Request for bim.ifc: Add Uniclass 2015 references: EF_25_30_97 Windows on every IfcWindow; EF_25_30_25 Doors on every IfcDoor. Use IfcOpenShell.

First a look at what the model holds.

```python
import ifcopenshell

model = ifcopenshell.open("bim.ifc")
print(model.schema)
print("classifications:", [c.Name for c in model.by_type("IfcClassification")])
for ifc_class in ("IfcDoor", "IfcRoof", "IfcStair", "IfcWall", "IfcWindow"):
    print(ifc_class, len(model.by_type(ifc_class)))
```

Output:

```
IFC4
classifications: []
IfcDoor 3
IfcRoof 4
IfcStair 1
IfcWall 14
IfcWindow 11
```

```python
import ifcopenshell
import ifcopenshell.api.classification

model = ifcopenshell.open("bim.ifc")

system = ifcopenshell.api.classification.add_classification(model, classification="Uniclass 2015")

codes = {
    "IfcWindow": ("EF_25_30_97", "Windows"),
    "IfcDoor": ("EF_25_30_25", "Doors"),
}
for ifc_class, (code, name) in codes.items():
    products = model.by_type(ifc_class)
    ifcopenshell.api.classification.add_reference(
        model, products=products, classification=system, identification=code, name=name
    )
    print(code, len(products))

model.write("bim-out.ifc")
```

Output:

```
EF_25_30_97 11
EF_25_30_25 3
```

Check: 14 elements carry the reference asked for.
